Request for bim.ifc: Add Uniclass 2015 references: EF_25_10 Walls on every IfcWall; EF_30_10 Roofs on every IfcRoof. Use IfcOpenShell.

First a look at what the model holds.

```python
import ifcopenshell

model = ifcopenshell.open("bim.ifc")
print(model.schema)
print("classifications:", [c.Name for c in model.by_type("IfcClassification")])
for ifc_class in ("IfcDoor", "IfcRoof", "IfcStair", "IfcWall", "IfcWindow"):
    print(ifc_class, len(model.by_type(ifc_class)))
```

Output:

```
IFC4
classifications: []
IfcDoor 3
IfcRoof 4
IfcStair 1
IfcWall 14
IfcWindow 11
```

```python
import ifcopenshell
import ifcopenshell.api.classification

model = ifcopenshell.open("bim.ifc")

system = ifcopenshell.api.classification.add_classification(model, classification="Uniclass 2015")

codes = {
    "IfcWall": ("EF_25_10", "Walls"),
    "IfcRoof": ("EF_30_10", "Roofs"),
}
for ifc_class, (code, name) in codes.items():
    products = model.by_type(ifc_class)
    ifcopenshell.api.classification.add_reference(
        model, products=products, classification=system, identification=code, name=name
    )
    print(code, len(products))

model.write("bim_updated.ifc")
```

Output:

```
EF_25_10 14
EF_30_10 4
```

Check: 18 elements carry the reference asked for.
